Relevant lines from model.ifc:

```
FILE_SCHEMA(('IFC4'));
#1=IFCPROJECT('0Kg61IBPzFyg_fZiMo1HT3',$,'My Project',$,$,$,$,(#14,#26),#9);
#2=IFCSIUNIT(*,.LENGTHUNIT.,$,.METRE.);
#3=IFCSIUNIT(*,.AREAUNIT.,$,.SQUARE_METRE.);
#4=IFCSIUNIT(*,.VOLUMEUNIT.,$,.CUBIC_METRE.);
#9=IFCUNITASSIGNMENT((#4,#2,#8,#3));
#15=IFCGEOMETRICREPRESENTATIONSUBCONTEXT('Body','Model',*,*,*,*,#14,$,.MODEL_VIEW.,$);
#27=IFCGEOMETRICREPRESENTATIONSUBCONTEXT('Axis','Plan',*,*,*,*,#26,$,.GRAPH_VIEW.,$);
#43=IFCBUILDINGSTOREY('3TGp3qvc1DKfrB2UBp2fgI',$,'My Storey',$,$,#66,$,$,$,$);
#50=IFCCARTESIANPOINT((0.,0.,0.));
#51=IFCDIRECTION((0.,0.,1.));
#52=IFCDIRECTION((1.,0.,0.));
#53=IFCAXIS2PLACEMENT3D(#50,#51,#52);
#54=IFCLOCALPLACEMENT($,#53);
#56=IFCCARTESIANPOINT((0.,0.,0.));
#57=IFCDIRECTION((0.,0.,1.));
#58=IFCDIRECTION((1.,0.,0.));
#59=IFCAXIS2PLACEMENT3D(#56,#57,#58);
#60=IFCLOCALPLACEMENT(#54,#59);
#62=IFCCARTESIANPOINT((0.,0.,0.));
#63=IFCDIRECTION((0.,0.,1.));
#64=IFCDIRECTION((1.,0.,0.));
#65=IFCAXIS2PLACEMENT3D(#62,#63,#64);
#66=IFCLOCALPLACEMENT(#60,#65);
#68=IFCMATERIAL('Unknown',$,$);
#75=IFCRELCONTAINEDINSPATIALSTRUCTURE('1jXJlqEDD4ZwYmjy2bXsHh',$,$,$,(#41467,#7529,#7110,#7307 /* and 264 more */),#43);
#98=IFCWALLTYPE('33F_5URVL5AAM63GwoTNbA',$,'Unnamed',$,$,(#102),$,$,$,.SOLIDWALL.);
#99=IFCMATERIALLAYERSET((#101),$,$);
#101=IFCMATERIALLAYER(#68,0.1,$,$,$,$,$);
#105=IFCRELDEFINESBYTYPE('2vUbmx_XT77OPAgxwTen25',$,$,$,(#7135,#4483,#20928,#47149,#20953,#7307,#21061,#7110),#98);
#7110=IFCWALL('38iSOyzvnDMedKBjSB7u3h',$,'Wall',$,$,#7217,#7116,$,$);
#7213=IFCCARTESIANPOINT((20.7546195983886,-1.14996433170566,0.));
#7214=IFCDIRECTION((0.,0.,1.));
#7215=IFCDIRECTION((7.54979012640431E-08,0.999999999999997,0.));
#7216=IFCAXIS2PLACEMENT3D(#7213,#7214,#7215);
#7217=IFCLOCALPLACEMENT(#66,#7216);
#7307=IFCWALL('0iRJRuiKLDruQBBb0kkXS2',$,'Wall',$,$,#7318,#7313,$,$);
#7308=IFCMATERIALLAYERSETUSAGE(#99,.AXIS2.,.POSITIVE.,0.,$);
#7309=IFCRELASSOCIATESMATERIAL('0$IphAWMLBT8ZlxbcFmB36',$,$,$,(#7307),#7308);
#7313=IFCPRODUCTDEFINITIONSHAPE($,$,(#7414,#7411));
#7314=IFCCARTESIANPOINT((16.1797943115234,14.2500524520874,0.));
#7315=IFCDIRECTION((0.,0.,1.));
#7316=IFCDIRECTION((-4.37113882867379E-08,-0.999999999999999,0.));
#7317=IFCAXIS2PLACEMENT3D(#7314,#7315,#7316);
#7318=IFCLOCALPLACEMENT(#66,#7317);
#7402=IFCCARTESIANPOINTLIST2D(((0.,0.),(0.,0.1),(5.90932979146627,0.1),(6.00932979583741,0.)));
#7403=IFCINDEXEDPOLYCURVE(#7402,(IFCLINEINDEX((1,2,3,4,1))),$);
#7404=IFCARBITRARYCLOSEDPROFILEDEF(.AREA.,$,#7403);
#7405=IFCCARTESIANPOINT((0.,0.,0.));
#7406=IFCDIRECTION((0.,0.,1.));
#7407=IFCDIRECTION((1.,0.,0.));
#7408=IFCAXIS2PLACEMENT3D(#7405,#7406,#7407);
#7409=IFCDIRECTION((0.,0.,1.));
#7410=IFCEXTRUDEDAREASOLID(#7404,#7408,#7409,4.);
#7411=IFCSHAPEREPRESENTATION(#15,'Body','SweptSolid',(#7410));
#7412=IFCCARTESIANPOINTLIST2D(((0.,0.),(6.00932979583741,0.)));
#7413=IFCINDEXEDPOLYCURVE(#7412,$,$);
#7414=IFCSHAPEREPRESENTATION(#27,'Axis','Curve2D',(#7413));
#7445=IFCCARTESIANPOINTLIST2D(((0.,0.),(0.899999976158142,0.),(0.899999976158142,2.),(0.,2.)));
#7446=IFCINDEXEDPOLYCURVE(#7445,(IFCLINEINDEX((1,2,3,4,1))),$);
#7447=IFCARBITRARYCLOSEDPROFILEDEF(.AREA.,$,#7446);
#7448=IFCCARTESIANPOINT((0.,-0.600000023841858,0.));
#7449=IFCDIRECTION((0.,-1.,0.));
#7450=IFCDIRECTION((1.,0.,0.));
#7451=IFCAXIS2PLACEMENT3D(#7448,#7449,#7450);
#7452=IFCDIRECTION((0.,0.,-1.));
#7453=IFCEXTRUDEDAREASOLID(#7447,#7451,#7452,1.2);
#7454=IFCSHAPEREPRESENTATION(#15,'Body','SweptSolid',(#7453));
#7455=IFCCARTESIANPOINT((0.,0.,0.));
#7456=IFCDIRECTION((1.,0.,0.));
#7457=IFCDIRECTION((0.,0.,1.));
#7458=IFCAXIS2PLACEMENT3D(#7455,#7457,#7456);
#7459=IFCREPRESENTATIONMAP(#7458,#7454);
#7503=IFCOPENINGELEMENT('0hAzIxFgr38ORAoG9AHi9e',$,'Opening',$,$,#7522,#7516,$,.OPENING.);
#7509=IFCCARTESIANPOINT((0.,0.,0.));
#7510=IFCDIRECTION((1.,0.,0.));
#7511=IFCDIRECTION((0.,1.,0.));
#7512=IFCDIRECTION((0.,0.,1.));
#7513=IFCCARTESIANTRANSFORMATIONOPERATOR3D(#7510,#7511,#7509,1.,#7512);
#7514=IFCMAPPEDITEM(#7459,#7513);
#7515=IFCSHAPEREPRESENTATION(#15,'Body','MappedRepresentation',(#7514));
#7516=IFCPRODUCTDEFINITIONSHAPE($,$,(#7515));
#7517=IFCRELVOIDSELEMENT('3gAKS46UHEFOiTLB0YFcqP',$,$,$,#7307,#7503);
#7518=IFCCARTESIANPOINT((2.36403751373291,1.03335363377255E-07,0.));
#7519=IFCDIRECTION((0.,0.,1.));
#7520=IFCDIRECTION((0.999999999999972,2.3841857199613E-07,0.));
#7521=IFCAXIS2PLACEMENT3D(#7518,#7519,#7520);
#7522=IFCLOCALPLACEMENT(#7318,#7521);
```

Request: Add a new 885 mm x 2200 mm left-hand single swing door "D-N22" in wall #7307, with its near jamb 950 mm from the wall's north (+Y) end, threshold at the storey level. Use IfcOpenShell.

```python
import numpy as np
import ifcopenshell
import ifcopenshell.api.feature
import ifcopenshell.api.geometry
import ifcopenshell.api.root
import ifcopenshell.api.spatial
import ifcopenshell.geom
import ifcopenshell.util.element
import ifcopenshell.util.placement
import ifcopenshell.util.representation
import ifcopenshell.util.shape
import ifcopenshell.util.unit

model = ifcopenshell.open("model.ifc")
unit_scale = ifcopenshell.util.unit.calculate_unit_scale(model)
settings = ifcopenshell.geom.settings()


def volume(element):
    """Net volume in cubic metres, openings subtracted."""
    shape = ifcopenshell.geom.create_shape(settings, element)
    return ifcopenshell.util.shape.get_volume(shape.geometry)


wall = model.by_guid("0iRJRuiKLDruQBBb0kkXS2")
storey = ifcopenshell.util.element.get_container(wall, ifc_class="IfcBuildingStorey")
context = ifcopenshell.util.representation.get_context(model, "Model", "Body", "MODEL_VIEW")
before = volume(wall)

width, height, from_end, sill = 0.885, 2.2, 0.95, 0.0  # metres

# The wall runs along its own X axis, and the end named is its -X end.
wall_shape = ifcopenshell.geom.create_shape(settings, wall)
x, y, z = ifcopenshell.util.shape.get_vertices(wall_shape.geometry).T
start = x.min() + from_end
face, thickness = float(y.min()), float(y.max() - y.min())
wall_matrix = ifcopenshell.util.placement.get_local_placement(wall.ObjectPlacement)
level = ifcopenshell.util.placement.get_local_placement(storey.ObjectPlacement)[2, 3]


def in_wall(x, y):
    """Placement at x, y metres in the wall's axes, at sill height."""
    matrix = wall_matrix.copy()
    matrix[:, 3] = wall_matrix @ np.array([x / unit_scale, y / unit_scale, 0.0, 1.0])
    matrix[2, 3] = level + sill / unit_scale
    return matrix


# Opening: a box that overshoots both wall faces by 50 mm.
opening = ifcopenshell.api.root.create_entity(model, ifc_class="IfcOpeningElement", predefined_type="OPENING")
box = ifcopenshell.api.geometry.add_wall_representation(
    model, context=context, length=width, height=height, thickness=thickness + 0.1
)
ifcopenshell.api.geometry.assign_representation(model, product=opening, representation=box)
ifcopenshell.api.geometry.edit_object_placement(model, product=opening, matrix=in_wall(start, face - 0.05), is_si=False)
ifcopenshell.api.feature.add_feature(model, feature=opening, element=wall)

door = ifcopenshell.api.root.create_entity(model, ifc_class="IfcDoor", name="D-N22", predefined_type="DOOR")
door.OverallWidth, door.OverallHeight = width / unit_scale, height / unit_scale
door.OperationType = "SINGLE_SWING_LEFT"
body = ifcopenshell.api.geometry.add_door_representation(
    model,
    context=context,
    overall_width=door.OverallWidth,
    overall_height=door.OverallHeight,
    operation_type="SINGLE_SWING_LEFT",
    lining_properties={"LiningDepth": thickness / unit_scale, "ThresholdDepth": thickness / unit_scale},
)
ifcopenshell.api.geometry.assign_representation(model, product=door, representation=body)
ifcopenshell.api.spatial.assign_container(model, products=[door], relating_structure=storey)
ifcopenshell.api.feature.add_filling(model, opening=opening, element=door)

# The lining spans the wall, so the door starts at the wall face.
ifcopenshell.api.geometry.edit_object_placement(model, product=door, matrix=in_wall(start, face), is_si=False)

after = volume(wall)

print(f"wall volume {before:.3f} -> {after:.3f} m3")

model.write("model_rev.ifc")
```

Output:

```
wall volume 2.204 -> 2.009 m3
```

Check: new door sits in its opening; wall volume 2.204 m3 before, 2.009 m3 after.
